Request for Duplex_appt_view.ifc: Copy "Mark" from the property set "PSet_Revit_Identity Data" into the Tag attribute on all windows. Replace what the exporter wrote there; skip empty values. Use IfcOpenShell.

First a look at what the model holds.

```python
import ifcopenshell
import ifcopenshell.util.element

model = ifcopenshell.open("Duplex_appt_view.ifc")
print(model.schema)
windows = model.by_type("IfcWindow")
print(len(windows), "windows")
for e in windows[:8]:
    source = ifcopenshell.util.element.get_pset(e, "PSet_Revit_Identity Data", "Mark")
    target = e.Tag
    print(e.id(), repr(source), repr(target), sep=" | ")
```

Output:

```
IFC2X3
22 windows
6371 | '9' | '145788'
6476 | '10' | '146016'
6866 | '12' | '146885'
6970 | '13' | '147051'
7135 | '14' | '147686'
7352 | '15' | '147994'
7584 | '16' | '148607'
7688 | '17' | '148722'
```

```python
import ifcopenshell
import ifcopenshell.util.element

model = ifcopenshell.open("Duplex_appt_view.ifc")

count = 0
for e in model.by_type("IfcWindow"):
    value = ifcopenshell.util.element.get_pset(e, "PSet_Revit_Identity Data", "Mark")
    current = e.Tag
    if not value or not value.strip() or current == value:
        continue
    e.Tag = value
    count += 1

print(count, "windows updated")

model.write("Duplex_appt_view_edited.ifc")
```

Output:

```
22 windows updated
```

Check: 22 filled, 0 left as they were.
